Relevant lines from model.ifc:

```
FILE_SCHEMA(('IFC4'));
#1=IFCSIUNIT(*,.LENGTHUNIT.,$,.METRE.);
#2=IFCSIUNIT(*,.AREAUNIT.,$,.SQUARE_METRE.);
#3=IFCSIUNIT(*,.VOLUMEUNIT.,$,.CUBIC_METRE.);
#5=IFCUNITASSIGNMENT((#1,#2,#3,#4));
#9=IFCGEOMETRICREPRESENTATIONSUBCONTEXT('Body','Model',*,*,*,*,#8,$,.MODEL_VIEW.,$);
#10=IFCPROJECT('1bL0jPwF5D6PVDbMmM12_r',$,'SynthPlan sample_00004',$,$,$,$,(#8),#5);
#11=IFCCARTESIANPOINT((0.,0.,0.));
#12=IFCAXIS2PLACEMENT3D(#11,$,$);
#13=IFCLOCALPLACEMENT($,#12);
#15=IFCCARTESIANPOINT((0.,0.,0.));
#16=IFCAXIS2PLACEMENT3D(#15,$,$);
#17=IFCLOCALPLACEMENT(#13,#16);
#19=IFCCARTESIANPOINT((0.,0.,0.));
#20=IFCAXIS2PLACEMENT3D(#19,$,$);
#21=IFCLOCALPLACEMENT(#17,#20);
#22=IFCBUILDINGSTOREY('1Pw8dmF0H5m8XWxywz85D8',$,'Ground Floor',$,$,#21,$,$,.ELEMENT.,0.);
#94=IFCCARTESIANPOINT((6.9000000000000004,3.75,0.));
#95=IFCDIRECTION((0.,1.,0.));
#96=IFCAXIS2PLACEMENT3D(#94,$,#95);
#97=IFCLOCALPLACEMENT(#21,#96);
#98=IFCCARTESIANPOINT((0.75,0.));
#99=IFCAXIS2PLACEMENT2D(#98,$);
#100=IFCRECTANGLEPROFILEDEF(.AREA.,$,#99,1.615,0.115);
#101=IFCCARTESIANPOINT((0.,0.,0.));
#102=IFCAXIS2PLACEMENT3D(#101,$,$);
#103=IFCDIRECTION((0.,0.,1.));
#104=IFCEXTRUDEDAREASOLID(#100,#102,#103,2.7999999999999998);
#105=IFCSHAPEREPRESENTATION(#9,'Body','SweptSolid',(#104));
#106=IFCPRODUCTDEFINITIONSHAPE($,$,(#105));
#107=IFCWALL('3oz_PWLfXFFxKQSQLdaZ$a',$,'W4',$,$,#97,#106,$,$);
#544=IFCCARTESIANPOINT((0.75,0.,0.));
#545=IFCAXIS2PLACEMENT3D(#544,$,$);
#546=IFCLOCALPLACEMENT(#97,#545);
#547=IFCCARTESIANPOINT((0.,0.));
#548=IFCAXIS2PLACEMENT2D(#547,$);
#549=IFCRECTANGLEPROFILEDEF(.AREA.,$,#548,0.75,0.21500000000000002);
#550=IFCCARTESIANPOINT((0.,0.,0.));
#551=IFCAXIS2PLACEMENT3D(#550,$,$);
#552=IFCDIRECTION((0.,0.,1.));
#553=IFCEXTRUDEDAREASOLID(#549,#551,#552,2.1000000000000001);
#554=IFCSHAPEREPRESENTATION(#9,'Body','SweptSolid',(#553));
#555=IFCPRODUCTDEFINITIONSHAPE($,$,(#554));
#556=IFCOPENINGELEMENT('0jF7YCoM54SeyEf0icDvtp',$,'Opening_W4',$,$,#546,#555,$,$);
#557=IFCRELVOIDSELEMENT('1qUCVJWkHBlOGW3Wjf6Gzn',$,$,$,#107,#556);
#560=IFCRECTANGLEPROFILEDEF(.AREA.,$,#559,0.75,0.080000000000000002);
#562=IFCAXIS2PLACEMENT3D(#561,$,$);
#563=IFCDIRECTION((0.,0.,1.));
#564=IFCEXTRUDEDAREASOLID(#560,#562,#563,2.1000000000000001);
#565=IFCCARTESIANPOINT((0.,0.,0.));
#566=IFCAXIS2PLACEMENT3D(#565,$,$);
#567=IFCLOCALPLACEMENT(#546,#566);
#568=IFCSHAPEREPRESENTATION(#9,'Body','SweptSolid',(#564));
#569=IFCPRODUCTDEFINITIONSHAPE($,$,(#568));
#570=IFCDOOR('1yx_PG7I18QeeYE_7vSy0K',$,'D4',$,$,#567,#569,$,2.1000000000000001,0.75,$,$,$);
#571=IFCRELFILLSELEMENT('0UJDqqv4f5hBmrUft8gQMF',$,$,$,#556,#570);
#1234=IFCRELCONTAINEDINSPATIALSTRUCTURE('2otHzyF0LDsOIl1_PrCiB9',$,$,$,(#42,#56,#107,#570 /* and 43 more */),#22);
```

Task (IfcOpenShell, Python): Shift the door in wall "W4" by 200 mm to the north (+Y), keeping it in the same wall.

```python
import ifcopenshell
import ifcopenshell.api.geometry
import ifcopenshell.util.placement
import ifcopenshell.util.unit

model = ifcopenshell.open("model.ifc")
unit_scale = ifcopenshell.util.unit.calculate_unit_scale(model)

door = model.by_id(570)
opening = door.FillsVoids[0].RelatingOpeningElement
wall = opening.VoidsElements[0].RelatingBuildingElement

wall_matrix = ifcopenshell.util.placement.get_local_placement(wall.ObjectPlacement)
shift = wall_matrix[:3, 0] * 0.2 / unit_scale
before = ifcopenshell.util.placement.get_local_placement(door.ObjectPlacement)[:3, 3].copy()

# The door is placed relative to its opening, so it follows when the opening moves.
matrix = ifcopenshell.util.placement.get_local_placement(opening.ObjectPlacement)
matrix[:3, 3] += shift
ifcopenshell.api.geometry.edit_object_placement(
    model, product=opening, matrix=matrix, is_si=False, should_transform_children=True
)

after = ifcopenshell.util.placement.get_local_placement(door.ObjectPlacement)[:3, 3]
print("door moved by", (after - before).round(3) + 0.0)

model.write("model_v2.ifc")
```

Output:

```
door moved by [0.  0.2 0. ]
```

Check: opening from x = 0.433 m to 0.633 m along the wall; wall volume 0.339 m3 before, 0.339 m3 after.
